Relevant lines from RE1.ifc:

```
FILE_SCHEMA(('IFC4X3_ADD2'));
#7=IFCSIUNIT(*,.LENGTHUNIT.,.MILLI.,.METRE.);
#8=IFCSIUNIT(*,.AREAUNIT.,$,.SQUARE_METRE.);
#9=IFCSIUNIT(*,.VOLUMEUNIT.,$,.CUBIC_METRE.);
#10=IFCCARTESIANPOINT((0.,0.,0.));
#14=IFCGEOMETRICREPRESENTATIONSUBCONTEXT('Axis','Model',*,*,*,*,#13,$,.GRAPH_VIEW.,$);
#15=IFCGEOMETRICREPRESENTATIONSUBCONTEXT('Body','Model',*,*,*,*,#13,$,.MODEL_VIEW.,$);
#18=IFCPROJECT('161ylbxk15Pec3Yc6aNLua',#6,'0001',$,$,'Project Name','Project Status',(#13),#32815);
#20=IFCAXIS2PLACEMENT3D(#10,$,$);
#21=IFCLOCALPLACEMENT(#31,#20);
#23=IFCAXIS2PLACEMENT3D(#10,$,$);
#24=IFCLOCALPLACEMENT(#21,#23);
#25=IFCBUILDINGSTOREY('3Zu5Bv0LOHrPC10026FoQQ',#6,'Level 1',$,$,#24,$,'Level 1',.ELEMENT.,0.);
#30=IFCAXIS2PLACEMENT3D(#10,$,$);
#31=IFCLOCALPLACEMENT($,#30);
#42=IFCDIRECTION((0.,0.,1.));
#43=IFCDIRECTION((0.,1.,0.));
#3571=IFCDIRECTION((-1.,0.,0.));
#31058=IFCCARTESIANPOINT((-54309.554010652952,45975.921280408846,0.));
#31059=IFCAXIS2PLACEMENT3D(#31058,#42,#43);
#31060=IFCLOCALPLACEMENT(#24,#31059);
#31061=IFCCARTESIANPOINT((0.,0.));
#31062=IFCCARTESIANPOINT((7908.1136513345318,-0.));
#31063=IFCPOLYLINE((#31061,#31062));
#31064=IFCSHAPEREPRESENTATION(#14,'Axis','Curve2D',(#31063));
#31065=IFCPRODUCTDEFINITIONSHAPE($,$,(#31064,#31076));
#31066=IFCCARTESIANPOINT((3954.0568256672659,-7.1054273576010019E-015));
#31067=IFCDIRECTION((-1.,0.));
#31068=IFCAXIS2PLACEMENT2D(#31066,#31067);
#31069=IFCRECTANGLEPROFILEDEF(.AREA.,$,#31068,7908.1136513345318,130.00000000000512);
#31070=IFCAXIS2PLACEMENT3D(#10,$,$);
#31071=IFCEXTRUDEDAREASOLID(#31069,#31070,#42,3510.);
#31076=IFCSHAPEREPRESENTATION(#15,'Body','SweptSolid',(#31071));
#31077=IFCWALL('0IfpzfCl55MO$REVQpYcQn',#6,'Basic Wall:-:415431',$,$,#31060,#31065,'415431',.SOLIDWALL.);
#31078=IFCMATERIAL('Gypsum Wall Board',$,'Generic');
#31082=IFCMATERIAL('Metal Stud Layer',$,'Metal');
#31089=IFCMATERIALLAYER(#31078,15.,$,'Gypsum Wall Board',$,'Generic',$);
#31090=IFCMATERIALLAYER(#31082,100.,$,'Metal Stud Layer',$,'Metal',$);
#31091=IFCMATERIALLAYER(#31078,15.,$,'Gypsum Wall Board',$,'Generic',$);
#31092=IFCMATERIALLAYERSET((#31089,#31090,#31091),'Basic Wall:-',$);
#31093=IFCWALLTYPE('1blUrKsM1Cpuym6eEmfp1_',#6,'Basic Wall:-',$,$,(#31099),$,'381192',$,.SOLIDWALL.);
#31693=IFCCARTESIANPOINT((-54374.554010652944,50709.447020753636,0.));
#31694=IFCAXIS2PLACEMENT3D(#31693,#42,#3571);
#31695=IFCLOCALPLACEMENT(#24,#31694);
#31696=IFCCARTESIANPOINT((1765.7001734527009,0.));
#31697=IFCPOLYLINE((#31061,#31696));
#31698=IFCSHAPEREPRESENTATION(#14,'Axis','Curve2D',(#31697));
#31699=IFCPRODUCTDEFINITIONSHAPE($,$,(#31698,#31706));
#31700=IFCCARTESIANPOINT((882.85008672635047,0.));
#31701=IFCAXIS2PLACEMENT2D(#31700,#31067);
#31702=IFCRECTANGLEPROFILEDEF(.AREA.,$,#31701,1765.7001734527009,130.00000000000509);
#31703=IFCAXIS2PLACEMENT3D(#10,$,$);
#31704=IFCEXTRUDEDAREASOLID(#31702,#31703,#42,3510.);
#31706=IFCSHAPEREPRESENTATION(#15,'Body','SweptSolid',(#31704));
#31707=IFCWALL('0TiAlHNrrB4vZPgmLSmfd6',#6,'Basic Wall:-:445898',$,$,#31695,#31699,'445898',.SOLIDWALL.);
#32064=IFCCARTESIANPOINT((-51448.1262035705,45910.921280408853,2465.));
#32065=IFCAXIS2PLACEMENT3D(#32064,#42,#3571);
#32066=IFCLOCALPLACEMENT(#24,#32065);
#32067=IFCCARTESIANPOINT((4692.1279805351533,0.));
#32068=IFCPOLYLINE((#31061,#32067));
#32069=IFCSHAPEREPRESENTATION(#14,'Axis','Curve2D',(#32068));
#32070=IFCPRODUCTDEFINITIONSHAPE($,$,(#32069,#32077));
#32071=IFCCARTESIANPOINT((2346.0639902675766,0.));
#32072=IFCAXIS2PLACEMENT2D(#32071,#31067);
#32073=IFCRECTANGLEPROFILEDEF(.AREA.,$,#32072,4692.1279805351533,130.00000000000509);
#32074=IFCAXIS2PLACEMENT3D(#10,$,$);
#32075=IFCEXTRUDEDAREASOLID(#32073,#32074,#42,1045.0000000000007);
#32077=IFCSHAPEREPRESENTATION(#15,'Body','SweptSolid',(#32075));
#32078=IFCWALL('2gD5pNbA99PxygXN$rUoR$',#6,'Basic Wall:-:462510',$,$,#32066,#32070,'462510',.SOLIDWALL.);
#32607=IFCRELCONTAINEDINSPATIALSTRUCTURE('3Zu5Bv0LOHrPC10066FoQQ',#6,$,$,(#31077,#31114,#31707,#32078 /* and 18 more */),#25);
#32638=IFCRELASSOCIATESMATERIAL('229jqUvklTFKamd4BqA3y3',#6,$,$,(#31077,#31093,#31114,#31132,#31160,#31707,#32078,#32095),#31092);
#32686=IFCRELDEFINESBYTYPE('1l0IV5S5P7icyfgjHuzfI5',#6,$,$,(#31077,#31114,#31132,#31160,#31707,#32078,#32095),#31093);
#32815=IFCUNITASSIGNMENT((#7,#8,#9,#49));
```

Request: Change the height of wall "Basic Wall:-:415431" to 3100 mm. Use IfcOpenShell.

```python
import ifcopenshell
import ifcopenshell.geom
import ifcopenshell.util.representation
import ifcopenshell.util.shape

model = ifcopenshell.open("RE1.ifc")
settings = ifcopenshell.geom.settings()


def volume(element):
    """Net volume in cubic metres, openings subtracted."""
    shape = ifcopenshell.geom.create_shape(settings, element)
    return ifcopenshell.util.shape.get_volume(shape.geometry)


wall = model.by_guid("0IfpzfCl55MO$REVQpYcQn")
before = volume(wall)

body = ifcopenshell.util.representation.get_representation(wall, "Model", "Body")
solid = body.Items[0]
old_height = solid.Depth
solid.Depth = 3100.0
after = volume(wall)

print(f"height {old_height:g} -> {solid.Depth:g}, volume {before:.3f} -> {after:.3f} m3")

model.write("RE1_updated.ifc")
```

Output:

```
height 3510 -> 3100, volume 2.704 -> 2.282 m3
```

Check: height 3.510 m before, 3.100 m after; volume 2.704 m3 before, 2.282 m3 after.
